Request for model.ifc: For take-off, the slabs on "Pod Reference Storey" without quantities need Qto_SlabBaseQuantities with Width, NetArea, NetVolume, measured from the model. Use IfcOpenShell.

First a look at what the model holds.

```python
import ifcopenshell
import ifcopenshell.util.element
import ifcopenshell.util.unit

model = ifcopenshell.open("model.ifc")
print(model.schema)
for unit_type in ("LENGTHUNIT", "AREAUNIT", "VOLUMEUNIT"):
    print(unit_type, ifcopenshell.util.unit.calculate_unit_scale(model, unit_type))
storey = next(s for s in model.by_type("IfcBuildingStorey") if s.Name == "Pod Reference Storey")
slabs = [e for e in ifcopenshell.util.element.get_decomposition(storey) if e.is_a("IfcSlab")]
for e in sorted(slabs, key=lambda e: e.id()):
    print(e.id(), e.is_a(), e.Name, list(ifcopenshell.util.element.get_psets(e, qtos_only=True)), sep=" | ")
```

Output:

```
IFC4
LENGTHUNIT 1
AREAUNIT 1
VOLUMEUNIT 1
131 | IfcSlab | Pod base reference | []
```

```python
import ifcopenshell
import ifcopenshell.api.pset
import ifcopenshell.geom
import ifcopenshell.util.element
import ifcopenshell.util.shape
import ifcopenshell.util.unit

model = ifcopenshell.open("model.ifc")
unit_scale = ifcopenshell.util.unit.calculate_unit_scale(model)
area_scale = ifcopenshell.util.unit.calculate_unit_scale(model, "AREAUNIT")
volume_scale = ifcopenshell.util.unit.calculate_unit_scale(model, "VOLUMEUNIT")
settings = ifcopenshell.geom.settings()

storey = next(s for s in model.by_type("IfcBuildingStorey") if s.Name == "Pod Reference Storey")
slabs = [e for e in ifcopenshell.util.element.get_decomposition(storey) if e.is_a("IfcSlab")]

for e in sorted(slabs, key=lambda e: e.id()):
    if ifcopenshell.util.element.get_psets(e, qtos_only=True, should_inherit=False):
        continue
    # Geometry comes back in metres, in the element's own axes.
    shape = ifcopenshell.geom.create_shape(settings, e)
    values = {
        "Width": ifcopenshell.util.shape.get_z(shape.geometry) / unit_scale,
        "NetArea": ifcopenshell.util.shape.get_footprint_area(shape.geometry) / area_scale,
        "NetVolume": ifcopenshell.util.shape.get_volume(shape.geometry) / volume_scale,
    }
    qto = ifcopenshell.api.pset.add_qto(model, product=e, name="Qto_SlabBaseQuantities")
    ifcopenshell.api.pset.edit_qto(model, qto=qto, properties=values)
    print(e.id(), {k: round(v, 3) for k, v in values.items()})

model.write("model_v2.ifc")
```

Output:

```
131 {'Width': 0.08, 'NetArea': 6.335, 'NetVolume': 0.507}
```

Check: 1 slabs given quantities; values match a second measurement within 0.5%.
